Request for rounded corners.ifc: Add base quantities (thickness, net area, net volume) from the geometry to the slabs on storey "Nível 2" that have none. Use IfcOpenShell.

First a look at what the model holds.

```python
import ifcopenshell
import ifcopenshell.util.element
import ifcopenshell.util.unit

model = ifcopenshell.open("rounded corners.ifc")
print(model.schema)
for unit_type in ("LENGTHUNIT", "AREAUNIT", "VOLUMEUNIT"):
    print(unit_type, ifcopenshell.util.unit.calculate_unit_scale(model, unit_type))
storey = next(s for s in model.by_type("IfcBuildingStorey") if s.Name == "Nível 2")
slabs = [e for e in ifcopenshell.util.element.get_decomposition(storey) if e.is_a("IfcSlab")]
for e in sorted(slabs, key=lambda e: e.id()):
    print(e.id(), e.is_a(), e.Name, list(ifcopenshell.util.element.get_psets(e, qtos_only=True)), sep=" | ")
```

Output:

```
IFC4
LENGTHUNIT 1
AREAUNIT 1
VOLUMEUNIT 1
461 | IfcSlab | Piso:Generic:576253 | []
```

```python
import ifcopenshell
import ifcopenshell.api.pset
import ifcopenshell.geom
import ifcopenshell.util.element
import ifcopenshell.util.shape
import ifcopenshell.util.unit

model = ifcopenshell.open("rounded corners.ifc")
unit_scale = ifcopenshell.util.unit.calculate_unit_scale(model)
area_scale = ifcopenshell.util.unit.calculate_unit_scale(model, "AREAUNIT")
volume_scale = ifcopenshell.util.unit.calculate_unit_scale(model, "VOLUMEUNIT")
settings = ifcopenshell.geom.settings()

storey = next(s for s in model.by_type("IfcBuildingStorey") if s.Name == "Nível 2")
slabs = [e for e in ifcopenshell.util.element.get_decomposition(storey) if e.is_a("IfcSlab")]

for e in sorted(slabs, key=lambda e: e.id()):
    if ifcopenshell.util.element.get_psets(e, qtos_only=True, should_inherit=False):
        continue
    # Geometry comes back in metres, in the element's own axes.
    shape = ifcopenshell.geom.create_shape(settings, e)
    values = {
        "Width": ifcopenshell.util.shape.get_z(shape.geometry) / unit_scale,
        "NetArea": ifcopenshell.util.shape.get_footprint_area(shape.geometry) / area_scale,
        "NetVolume": ifcopenshell.util.shape.get_volume(shape.geometry) / volume_scale,
    }
    qto = ifcopenshell.api.pset.add_qto(model, product=e, name="Qto_SlabBaseQuantities")
    ifcopenshell.api.pset.edit_qto(model, qto=qto, properties=values)
    print(e.id(), {k: round(v, 3) for k, v in values.items()})

model.write("rounded corners_v2.ifc")
```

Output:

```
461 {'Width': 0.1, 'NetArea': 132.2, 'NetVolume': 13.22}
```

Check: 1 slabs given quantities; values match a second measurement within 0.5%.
